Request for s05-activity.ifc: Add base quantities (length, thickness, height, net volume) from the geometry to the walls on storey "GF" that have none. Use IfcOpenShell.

First a look at what the model holds.

```python
import ifcopenshell
import ifcopenshell.util.element
import ifcopenshell.util.unit

model = ifcopenshell.open("s05-activity.ifc")
print(model.schema)
for unit_type in ("LENGTHUNIT", "AREAUNIT", "VOLUMEUNIT"):
    print(unit_type, ifcopenshell.util.unit.calculate_unit_scale(model, unit_type))
storey = next(s for s in model.by_type("IfcBuildingStorey") if s.Name == "GF")
walls = [e for e in ifcopenshell.util.element.get_decomposition(storey) if e.is_a("IfcWall")]
for e in sorted(walls, key=lambda e: e.id()):
    print(e.id(), e.is_a(), e.Name, list(ifcopenshell.util.element.get_psets(e, qtos_only=True)), sep=" | ")
```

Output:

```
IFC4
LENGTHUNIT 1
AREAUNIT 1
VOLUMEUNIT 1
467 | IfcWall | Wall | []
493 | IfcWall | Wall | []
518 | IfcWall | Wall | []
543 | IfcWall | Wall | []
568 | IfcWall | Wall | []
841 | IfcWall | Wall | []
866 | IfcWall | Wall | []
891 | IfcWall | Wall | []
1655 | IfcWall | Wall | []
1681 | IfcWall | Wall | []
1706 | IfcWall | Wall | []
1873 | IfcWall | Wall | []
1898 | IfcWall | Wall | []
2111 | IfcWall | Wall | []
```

```python
import ifcopenshell
import ifcopenshell.api.pset
import ifcopenshell.geom
import ifcopenshell.util.element
import ifcopenshell.util.shape
import ifcopenshell.util.unit

model = ifcopenshell.open("s05-activity.ifc")
unit_scale = ifcopenshell.util.unit.calculate_unit_scale(model)
volume_scale = ifcopenshell.util.unit.calculate_unit_scale(model, "VOLUMEUNIT")
settings = ifcopenshell.geom.settings()

storey = next(s for s in model.by_type("IfcBuildingStorey") if s.Name == "GF")
walls = [e for e in ifcopenshell.util.element.get_decomposition(storey) if e.is_a("IfcWall")]

for e in sorted(walls, key=lambda e: e.id()):
    if ifcopenshell.util.element.get_psets(e, qtos_only=True, should_inherit=False):
        continue
    # Geometry comes back in metres, in the element's own axes.
    shape = ifcopenshell.geom.create_shape(settings, e)
    values = {
        "Length": ifcopenshell.util.shape.get_x(shape.geometry) / unit_scale,
        "Width": ifcopenshell.util.shape.get_y(shape.geometry) / unit_scale,
        "Height": ifcopenshell.util.shape.get_z(shape.geometry) / unit_scale,
        "NetVolume": ifcopenshell.util.shape.get_volume(shape.geometry) / volume_scale,
    }
    qto = ifcopenshell.api.pset.add_qto(model, product=e, name="Qto_WallBaseQuantities")
    ifcopenshell.api.pset.edit_qto(model, qto=qto, properties=values)
    print(e.id(), {k: round(v, 3) for k, v in values.items()})

model.write("s05-activity_updated.ifc")
```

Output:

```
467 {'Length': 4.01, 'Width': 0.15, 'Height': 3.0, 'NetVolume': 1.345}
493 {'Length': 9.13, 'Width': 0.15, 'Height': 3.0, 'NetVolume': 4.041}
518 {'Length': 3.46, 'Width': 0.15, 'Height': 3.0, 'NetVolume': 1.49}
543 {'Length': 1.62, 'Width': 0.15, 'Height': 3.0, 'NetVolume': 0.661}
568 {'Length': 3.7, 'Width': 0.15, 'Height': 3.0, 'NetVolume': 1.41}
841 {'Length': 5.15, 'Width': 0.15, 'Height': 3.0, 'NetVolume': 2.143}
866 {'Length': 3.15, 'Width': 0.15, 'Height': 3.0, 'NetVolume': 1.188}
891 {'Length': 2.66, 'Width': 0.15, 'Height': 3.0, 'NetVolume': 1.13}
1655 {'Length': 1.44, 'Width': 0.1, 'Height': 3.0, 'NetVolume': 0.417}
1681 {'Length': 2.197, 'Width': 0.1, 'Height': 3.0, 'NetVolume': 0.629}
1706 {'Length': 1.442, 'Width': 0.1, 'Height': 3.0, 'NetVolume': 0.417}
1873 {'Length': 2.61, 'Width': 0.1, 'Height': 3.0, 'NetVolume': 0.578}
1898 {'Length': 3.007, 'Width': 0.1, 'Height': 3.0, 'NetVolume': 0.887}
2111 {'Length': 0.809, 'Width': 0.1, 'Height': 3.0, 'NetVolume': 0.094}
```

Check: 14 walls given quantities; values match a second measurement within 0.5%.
